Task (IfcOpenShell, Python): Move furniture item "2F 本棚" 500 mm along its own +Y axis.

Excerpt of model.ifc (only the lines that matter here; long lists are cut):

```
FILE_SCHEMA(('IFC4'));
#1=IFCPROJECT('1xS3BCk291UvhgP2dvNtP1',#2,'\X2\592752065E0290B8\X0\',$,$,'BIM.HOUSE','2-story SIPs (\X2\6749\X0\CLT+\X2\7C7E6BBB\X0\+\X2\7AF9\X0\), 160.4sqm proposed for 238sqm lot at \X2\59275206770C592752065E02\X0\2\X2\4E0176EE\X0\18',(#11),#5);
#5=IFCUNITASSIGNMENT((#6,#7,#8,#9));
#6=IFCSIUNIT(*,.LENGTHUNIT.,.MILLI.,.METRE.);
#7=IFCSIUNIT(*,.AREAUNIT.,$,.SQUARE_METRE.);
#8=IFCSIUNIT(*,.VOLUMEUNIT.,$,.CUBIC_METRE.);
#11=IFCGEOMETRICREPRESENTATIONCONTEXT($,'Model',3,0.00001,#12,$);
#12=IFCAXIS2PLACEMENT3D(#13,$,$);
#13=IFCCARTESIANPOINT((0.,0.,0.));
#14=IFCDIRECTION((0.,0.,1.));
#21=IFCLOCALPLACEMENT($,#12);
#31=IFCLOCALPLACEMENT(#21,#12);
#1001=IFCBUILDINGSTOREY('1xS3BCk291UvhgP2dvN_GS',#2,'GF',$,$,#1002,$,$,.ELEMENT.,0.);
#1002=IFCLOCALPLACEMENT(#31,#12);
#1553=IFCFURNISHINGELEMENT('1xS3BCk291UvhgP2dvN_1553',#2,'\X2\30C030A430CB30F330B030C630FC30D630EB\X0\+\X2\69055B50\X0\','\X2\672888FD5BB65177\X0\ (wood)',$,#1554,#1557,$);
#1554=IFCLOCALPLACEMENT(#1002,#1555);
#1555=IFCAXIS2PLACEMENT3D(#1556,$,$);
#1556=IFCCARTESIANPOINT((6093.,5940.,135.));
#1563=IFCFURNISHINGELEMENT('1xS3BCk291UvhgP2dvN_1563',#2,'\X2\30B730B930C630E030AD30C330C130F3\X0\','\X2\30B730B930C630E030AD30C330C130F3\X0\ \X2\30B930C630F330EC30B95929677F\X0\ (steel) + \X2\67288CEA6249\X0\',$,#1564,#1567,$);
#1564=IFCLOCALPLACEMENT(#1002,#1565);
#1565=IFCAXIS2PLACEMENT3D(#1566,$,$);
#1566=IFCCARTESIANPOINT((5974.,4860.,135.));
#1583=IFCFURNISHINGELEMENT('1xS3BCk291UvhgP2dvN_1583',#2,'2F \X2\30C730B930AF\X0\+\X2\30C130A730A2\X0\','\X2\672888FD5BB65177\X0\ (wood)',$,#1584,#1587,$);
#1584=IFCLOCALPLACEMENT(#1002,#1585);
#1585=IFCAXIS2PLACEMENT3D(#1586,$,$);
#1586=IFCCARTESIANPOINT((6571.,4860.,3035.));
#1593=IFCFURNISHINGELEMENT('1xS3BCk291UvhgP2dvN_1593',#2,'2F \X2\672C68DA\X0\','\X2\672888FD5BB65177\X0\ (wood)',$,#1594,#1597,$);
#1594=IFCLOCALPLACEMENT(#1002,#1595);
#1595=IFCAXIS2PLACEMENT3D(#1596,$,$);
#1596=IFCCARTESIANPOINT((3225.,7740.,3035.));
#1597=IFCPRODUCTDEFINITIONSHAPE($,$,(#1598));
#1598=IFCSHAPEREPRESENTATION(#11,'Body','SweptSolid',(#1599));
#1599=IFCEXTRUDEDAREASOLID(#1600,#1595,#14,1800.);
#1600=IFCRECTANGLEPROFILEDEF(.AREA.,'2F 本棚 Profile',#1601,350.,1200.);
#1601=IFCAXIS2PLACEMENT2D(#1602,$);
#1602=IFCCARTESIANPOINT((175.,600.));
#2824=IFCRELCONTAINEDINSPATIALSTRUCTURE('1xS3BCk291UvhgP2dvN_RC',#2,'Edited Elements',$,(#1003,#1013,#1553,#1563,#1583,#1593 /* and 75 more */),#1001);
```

```python
import ifcopenshell
import ifcopenshell.api.geometry
import ifcopenshell.util.placement

model = ifcopenshell.open("model.ifc")

item = model.by_guid("1xS3BCk291UvhgP2dvN_1593")
matrix = ifcopenshell.util.placement.get_local_placement(item.ObjectPlacement)
matrix[:3, 3] += matrix[:3, 1] * 500.0
ifcopenshell.api.geometry.edit_object_placement(model, product=item, matrix=matrix, is_si=False)

print(ifcopenshell.util.placement.get_local_placement(item.ObjectPlacement).round(3) + 0.0)

model.write("model_updated.ifc")
```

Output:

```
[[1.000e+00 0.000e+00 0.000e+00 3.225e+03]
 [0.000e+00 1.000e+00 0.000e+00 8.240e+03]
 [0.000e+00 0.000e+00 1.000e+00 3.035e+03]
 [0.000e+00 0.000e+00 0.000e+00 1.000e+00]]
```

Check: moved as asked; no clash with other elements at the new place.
